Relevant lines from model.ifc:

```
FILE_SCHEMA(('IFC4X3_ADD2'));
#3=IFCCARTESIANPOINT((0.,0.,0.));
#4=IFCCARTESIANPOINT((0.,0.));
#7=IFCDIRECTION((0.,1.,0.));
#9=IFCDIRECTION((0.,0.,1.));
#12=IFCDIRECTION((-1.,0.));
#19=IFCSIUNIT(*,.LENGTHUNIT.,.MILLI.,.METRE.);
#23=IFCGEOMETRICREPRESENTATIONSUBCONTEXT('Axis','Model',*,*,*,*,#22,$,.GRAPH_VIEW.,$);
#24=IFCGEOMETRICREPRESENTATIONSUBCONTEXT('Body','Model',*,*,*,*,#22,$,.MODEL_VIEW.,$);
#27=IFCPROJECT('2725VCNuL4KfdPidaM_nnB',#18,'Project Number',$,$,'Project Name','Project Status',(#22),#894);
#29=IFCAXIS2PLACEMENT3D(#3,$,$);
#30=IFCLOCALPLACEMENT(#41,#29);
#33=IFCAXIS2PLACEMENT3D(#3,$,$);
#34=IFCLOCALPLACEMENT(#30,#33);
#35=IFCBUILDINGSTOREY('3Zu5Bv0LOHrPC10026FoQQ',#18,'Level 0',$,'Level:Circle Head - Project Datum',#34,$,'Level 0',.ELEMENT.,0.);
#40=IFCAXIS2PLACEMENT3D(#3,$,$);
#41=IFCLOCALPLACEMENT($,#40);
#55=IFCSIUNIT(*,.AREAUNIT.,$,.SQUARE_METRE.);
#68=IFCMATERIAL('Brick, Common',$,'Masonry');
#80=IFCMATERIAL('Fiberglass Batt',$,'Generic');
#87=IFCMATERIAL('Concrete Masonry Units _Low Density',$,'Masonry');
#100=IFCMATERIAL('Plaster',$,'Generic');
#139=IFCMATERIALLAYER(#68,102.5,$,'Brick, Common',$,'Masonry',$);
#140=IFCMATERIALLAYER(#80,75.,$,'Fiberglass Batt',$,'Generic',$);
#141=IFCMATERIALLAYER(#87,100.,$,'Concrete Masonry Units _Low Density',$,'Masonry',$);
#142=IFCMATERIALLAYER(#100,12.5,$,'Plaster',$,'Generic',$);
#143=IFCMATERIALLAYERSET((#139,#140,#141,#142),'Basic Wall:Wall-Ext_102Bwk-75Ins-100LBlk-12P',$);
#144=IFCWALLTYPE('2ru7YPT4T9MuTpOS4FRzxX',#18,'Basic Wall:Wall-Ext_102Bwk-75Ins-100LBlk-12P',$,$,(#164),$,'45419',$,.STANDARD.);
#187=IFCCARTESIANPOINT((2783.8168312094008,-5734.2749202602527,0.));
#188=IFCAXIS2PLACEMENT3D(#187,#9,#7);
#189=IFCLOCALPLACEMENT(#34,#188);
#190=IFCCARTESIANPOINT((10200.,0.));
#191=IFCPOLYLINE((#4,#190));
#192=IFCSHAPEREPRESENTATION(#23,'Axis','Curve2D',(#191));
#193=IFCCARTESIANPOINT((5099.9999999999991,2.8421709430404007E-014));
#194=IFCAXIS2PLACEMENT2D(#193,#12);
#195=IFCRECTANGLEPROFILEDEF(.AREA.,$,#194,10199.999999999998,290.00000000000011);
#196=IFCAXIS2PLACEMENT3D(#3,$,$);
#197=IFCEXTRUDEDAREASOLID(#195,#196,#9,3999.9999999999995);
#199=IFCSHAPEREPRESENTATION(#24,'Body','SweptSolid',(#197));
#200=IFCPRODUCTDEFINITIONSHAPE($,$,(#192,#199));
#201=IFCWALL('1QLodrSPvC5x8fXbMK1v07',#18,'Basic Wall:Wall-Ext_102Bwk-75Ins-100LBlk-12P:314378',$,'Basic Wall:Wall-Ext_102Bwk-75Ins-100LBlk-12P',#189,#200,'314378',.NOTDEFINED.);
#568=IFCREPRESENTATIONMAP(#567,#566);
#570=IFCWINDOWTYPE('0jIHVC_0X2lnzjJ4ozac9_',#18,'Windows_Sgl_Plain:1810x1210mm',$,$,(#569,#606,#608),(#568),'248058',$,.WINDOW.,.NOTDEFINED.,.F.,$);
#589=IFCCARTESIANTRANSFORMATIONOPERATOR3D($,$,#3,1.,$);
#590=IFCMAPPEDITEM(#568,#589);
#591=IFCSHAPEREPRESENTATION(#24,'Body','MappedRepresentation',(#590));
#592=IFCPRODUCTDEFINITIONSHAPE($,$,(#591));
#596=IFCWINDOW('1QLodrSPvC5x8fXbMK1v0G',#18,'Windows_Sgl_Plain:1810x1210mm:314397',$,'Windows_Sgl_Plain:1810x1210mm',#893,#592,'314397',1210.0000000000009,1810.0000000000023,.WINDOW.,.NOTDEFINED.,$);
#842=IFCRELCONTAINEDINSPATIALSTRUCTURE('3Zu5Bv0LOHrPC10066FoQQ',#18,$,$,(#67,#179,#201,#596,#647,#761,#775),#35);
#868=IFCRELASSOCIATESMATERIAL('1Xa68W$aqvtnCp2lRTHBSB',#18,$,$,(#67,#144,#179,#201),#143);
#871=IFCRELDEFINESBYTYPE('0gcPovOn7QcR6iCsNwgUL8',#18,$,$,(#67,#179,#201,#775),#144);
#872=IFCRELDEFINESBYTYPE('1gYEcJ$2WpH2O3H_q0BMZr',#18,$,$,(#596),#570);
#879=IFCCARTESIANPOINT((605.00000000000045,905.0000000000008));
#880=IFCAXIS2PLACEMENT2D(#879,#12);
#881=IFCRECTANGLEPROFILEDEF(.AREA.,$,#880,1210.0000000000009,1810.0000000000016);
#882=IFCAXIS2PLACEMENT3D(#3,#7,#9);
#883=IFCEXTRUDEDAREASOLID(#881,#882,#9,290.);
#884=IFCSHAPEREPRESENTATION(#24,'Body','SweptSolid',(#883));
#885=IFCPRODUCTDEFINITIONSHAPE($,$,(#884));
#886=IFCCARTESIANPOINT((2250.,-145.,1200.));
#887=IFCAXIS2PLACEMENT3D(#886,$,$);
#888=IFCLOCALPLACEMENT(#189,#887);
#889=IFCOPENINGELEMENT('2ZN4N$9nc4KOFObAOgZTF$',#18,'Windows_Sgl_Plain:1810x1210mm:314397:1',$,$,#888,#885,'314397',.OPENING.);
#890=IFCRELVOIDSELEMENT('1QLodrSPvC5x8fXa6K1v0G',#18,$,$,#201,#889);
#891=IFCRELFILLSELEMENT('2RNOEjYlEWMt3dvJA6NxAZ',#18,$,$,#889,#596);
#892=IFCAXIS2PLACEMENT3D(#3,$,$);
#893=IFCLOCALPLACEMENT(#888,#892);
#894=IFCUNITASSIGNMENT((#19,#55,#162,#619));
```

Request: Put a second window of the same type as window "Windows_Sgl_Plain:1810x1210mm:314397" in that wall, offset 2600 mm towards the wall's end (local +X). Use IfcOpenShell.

```python
import ifcopenshell
import ifcopenshell.api.feature
import ifcopenshell.api.geometry
import ifcopenshell.api.root
import ifcopenshell.geom
import ifcopenshell.util.element
import ifcopenshell.util.placement
import ifcopenshell.util.shape

model = ifcopenshell.open("model.ifc")
settings = ifcopenshell.geom.settings()


def volume(element):
    """Net volume in cubic metres, openings subtracted."""
    shape = ifcopenshell.geom.create_shape(settings, element)
    return ifcopenshell.util.shape.get_volume(shape.geometry)


def reuse_history(source, copy):
    """copy_class also copies each property set's owner history, people and application; keep the originals."""
    for rel in copy.IsDefinedBy:
        if rel.is_a("IfcRelDefinesByProperties") and (history := rel.RelatingPropertyDefinition.OwnerHistory):
            rel.RelatingPropertyDefinition.OwnerHistory = source.OwnerHistory
            ifcopenshell.util.element.remove_deep2(model, history)


window = model.by_guid("1QLodrSPvC5x8fXbMK1v0G")
opening = window.FillsVoids[0].RelatingOpeningElement
wall = opening.VoidsElements[0].RelatingBuildingElement
before = volume(wall)
shift = ifcopenshell.util.placement.get_local_placement(wall.ObjectPlacement)[:3, 0] * 2600.0

# copy_class copies the void relationship, type, container and properties, but no geometry.
new_opening = ifcopenshell.api.root.copy_class(model, product=opening)
new_opening.Representation = ifcopenshell.util.element.copy_deep(
    model, opening.Representation, exclude=["IfcGeometricRepresentationContext", "IfcRepresentationMap"]
)
new_opening.Name = "Windows_Sgl_Plain:1810x1210mm"
new_opening.Tag = None
new_window = ifcopenshell.api.root.copy_class(model, product=window)
new_window.Representation = ifcopenshell.util.element.copy_deep(
    model, window.Representation, exclude=["IfcGeometricRepresentationContext", "IfcRepresentationMap"]
)
new_window.Name = "Windows_Sgl_Plain:1810x1210mm"
new_window.Tag = None
reuse_history(window, new_window)
ifcopenshell.api.feature.add_filling(model, opening=new_opening, element=new_window)

for old, new in ((opening, new_opening), (window, new_window)):
    matrix = ifcopenshell.util.placement.get_local_placement(old.ObjectPlacement)
    matrix[:3, 3] += shift
    ifcopenshell.api.geometry.edit_object_placement(model, product=new, matrix=matrix, is_si=False)

after = volume(wall)

print(f"wall volume {before:.3f} -> {after:.3f} m3")

model.write("model_rev.ifc")
```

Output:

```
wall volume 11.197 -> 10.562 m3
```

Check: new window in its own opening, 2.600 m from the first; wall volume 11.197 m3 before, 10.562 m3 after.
